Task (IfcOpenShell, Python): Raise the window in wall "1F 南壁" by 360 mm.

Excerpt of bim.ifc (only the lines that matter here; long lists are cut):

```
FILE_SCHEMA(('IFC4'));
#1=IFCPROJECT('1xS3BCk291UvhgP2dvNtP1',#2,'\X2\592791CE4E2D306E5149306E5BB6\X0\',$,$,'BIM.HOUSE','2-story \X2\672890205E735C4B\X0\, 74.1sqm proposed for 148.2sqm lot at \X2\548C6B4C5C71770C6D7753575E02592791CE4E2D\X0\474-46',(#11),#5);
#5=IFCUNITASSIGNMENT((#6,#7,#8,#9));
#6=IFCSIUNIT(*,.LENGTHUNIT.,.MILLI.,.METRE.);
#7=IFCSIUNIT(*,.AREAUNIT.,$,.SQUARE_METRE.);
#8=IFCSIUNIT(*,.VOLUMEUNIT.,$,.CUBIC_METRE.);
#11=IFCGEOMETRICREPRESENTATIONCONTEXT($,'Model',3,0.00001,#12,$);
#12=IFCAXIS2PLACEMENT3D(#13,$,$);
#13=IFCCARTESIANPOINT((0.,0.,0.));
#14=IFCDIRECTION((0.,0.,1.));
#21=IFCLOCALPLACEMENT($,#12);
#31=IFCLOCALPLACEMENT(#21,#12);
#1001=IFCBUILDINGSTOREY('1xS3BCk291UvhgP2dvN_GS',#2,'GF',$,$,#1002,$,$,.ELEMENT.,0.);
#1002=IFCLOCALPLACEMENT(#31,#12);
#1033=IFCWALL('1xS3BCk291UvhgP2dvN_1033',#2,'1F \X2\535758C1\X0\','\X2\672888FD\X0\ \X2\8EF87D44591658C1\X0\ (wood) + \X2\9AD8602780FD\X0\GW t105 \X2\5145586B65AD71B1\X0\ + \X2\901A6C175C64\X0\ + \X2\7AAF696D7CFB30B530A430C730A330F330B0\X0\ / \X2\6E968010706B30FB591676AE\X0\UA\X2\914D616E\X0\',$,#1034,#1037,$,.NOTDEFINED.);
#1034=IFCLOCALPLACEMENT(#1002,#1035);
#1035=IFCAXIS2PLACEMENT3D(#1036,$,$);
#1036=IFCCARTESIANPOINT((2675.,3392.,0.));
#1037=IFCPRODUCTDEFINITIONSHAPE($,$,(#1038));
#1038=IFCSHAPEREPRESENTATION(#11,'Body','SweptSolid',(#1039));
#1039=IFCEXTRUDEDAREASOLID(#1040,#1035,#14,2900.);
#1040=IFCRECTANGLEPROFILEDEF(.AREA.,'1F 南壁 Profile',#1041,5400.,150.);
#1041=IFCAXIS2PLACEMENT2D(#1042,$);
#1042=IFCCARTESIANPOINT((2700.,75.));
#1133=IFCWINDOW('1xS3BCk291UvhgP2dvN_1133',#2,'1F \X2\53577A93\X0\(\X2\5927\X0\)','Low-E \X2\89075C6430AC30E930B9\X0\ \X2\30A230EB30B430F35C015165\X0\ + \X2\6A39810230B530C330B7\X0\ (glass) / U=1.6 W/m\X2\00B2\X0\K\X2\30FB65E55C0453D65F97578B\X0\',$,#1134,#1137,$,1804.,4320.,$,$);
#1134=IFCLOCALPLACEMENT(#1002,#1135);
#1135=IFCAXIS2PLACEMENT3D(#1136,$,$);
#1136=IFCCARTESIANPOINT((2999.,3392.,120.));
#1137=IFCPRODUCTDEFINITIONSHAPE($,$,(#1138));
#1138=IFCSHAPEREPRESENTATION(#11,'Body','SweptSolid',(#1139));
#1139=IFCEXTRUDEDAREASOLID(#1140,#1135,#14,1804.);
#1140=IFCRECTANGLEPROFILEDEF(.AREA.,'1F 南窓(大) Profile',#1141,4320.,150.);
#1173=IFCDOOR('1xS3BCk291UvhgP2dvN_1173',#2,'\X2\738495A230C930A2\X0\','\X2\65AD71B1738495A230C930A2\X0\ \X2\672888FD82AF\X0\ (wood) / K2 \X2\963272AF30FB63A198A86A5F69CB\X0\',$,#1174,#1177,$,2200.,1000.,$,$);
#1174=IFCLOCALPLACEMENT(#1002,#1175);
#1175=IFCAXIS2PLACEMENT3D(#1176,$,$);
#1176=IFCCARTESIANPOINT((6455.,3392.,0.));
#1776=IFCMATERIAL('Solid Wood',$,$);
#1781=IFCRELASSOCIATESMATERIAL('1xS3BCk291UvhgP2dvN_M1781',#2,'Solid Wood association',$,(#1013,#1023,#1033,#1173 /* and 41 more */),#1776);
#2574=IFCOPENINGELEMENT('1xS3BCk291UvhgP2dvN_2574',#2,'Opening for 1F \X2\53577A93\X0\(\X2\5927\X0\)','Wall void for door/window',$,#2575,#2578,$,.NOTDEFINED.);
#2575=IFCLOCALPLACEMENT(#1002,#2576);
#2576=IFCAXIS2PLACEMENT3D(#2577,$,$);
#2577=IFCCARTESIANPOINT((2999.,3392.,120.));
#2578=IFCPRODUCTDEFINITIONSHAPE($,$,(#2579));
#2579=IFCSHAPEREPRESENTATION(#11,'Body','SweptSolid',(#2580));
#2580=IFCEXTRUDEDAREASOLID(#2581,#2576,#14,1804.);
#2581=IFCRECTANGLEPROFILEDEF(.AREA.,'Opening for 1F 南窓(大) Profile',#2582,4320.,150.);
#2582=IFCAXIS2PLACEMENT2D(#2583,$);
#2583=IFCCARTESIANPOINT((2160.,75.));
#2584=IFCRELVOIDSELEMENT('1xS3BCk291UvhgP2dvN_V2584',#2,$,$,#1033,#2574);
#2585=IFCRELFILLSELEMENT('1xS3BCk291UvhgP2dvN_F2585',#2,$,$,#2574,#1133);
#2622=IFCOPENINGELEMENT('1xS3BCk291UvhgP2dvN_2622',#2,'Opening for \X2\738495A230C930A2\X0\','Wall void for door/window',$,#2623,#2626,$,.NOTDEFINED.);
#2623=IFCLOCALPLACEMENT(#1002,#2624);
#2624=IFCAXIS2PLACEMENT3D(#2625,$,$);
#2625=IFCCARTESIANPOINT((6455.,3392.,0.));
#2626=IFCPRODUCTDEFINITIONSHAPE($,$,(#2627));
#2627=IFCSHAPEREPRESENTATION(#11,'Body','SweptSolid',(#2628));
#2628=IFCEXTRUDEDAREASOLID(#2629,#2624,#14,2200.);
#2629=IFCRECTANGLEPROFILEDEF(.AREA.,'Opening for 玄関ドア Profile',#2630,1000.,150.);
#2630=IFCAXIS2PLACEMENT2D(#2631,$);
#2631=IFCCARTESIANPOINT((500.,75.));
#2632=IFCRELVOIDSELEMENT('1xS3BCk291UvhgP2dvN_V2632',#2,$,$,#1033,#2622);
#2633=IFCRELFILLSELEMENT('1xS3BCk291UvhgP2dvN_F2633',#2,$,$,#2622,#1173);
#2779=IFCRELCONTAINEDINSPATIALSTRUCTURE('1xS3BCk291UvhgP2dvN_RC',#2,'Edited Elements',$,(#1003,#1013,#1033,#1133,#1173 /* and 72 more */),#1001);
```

```python
import numpy as np
import ifcopenshell
import ifcopenshell.api.geometry
import ifcopenshell.util.placement
import ifcopenshell.util.unit

model = ifcopenshell.open("bim.ifc")
unit_scale = ifcopenshell.util.unit.calculate_unit_scale(model)

window = model.by_guid("1xS3BCk291UvhgP2dvN_1133")
opening = window.FillsVoids[0].RelatingOpeningElement
dz = 0.36 / unit_scale

shift = np.array([0.0, 0.0, dz])
# The window is not placed relative to its opening, so move both.
for product in (opening, window):
    matrix = ifcopenshell.util.placement.get_local_placement(product.ObjectPlacement)
    matrix[:3, 3] += shift
    ifcopenshell.api.geometry.edit_object_placement(model, product=product, matrix=matrix, is_si=False)

print(f"moved by {dz * unit_scale:+.3f} m")

model.write("bim_updated.ifc")
```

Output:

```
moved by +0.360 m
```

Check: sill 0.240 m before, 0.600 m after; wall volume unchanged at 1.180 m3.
